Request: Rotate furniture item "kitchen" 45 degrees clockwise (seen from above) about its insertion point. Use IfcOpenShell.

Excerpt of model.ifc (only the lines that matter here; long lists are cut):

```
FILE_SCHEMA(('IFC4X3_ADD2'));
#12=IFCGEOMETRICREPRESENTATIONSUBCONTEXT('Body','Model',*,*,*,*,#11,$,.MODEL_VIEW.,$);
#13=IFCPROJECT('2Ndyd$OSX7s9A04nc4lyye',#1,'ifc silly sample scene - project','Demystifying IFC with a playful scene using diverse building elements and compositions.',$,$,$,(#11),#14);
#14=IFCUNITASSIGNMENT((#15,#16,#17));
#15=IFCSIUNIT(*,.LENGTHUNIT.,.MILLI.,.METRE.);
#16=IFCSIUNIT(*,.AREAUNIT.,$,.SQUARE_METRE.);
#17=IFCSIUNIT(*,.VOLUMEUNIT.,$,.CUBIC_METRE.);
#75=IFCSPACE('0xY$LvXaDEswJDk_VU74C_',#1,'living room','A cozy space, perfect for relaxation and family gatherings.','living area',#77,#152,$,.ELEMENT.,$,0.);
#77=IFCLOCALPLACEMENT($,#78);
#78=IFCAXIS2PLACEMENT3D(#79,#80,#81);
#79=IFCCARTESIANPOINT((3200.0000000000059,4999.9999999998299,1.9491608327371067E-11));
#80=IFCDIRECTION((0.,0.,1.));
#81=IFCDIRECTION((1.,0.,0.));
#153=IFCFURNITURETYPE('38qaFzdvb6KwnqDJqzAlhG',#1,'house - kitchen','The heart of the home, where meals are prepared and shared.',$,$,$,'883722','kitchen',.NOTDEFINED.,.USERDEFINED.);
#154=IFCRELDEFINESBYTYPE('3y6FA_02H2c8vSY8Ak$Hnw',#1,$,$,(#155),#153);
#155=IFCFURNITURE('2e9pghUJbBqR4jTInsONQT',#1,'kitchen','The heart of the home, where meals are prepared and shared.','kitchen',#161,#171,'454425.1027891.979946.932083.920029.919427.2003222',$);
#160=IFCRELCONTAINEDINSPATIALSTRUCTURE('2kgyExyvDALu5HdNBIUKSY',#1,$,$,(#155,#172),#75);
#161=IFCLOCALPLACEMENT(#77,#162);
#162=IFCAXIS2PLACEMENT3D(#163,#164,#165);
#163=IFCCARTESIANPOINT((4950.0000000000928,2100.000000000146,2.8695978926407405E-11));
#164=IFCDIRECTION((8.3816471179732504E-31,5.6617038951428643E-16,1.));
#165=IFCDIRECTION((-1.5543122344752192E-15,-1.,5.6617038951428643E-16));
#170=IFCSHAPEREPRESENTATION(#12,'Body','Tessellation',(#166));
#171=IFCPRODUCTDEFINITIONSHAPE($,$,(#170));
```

```python
import ifcopenshell
import ifcopenshell.api.geometry
import ifcopenshell.util.placement

model = ifcopenshell.open("model.ifc")

item = model.by_guid("2e9pghUJbBqR4jTInsONQT")
matrix = ifcopenshell.util.placement.get_local_placement(item.ObjectPlacement)
matrix = matrix @ ifcopenshell.util.placement.rotation(-45, "Z")
ifcopenshell.api.geometry.edit_object_placement(model, product=item, matrix=matrix, is_si=False)

print(ifcopenshell.util.placement.get_local_placement(item.ObjectPlacement).round(3) + 0.0)

model.write("model_rev.ifc")
```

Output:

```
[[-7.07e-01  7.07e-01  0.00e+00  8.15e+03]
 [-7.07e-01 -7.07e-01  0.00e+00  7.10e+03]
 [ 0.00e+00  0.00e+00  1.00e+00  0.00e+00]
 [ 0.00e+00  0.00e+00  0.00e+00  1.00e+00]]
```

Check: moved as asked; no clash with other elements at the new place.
